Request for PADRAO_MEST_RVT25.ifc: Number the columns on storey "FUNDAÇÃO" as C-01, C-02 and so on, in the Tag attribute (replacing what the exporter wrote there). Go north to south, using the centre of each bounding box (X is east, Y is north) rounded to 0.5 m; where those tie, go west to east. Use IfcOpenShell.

First a look at what the model holds.

```python
import ifcopenshell
import ifcopenshell.util.element
import ifcopenshell.util.placement

model = ifcopenshell.open("PADRAO_MEST_RVT25.ifc")
print(model.schema)
storey = next(s for s in model.by_type("IfcBuildingStorey") if s.Name == "FUNDAÇÃO")
columns = [e for e in ifcopenshell.util.element.get_decomposition(storey) if e.is_a("IfcColumn")]
for e in sorted(columns, key=lambda e: e.id()):
    origin = ifcopenshell.util.placement.get_local_placement(e.ObjectPlacement)[:3, 3]
    print(e.id(), e.Tag, e.Name, origin.round(2) + 0.0, sep=" | ")
```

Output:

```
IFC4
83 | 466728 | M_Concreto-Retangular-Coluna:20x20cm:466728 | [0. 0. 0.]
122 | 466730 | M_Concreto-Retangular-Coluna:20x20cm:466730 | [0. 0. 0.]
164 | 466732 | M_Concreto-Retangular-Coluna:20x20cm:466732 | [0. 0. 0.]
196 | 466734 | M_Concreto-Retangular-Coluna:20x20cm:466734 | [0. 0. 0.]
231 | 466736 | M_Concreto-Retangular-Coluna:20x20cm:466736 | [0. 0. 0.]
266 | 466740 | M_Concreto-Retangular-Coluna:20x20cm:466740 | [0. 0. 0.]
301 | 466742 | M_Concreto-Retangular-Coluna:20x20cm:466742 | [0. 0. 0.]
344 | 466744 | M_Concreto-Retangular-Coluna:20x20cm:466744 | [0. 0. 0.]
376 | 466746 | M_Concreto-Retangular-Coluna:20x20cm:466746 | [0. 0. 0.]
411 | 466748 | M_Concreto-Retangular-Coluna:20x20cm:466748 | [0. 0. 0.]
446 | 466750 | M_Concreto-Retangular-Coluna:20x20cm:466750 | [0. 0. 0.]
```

```python
import ifcopenshell
import ifcopenshell.geom
import ifcopenshell.util.element
import ifcopenshell.util.shape

model = ifcopenshell.open("PADRAO_MEST_RVT25.ifc")
settings = ifcopenshell.geom.settings()
settings.set("use-world-coords", True)


def centre(element):
    shape = ifcopenshell.geom.create_shape(settings, element)
    return ifcopenshell.util.shape.get_bbox_centroid(shape.geometry)


storey = next(s for s in model.by_type("IfcBuildingStorey") if s.Name == "FUNDAÇÃO")
columns = [e for e in ifcopenshell.util.element.get_decomposition(storey) if e.is_a("IfcColumn")]

# Insertion points can sit at a corner or the storey origin, so sort by the geometry (in metres).
centres = {e: centre(e) for e in columns}
columns.sort(key=lambda e: (-round(centres[e][1] / 0.5), centres[e][0]))

for i, e in enumerate(columns, start=1):
    number = f"C-{i:02d}"
    e.Tag = number
    print(e.id(), number)

model.write("PADRAO_MEST_RVT25_updated.ifc")
```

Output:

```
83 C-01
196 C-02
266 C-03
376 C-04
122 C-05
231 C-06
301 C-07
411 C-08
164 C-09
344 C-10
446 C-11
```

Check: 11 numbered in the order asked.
